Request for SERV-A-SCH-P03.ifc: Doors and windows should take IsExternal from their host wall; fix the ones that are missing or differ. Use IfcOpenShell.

First a look at what the model holds.

```python
import ifcopenshell
import ifcopenshell.util.element

model = ifcopenshell.open("SERV-A-SCH-P03.ifc")
print(model.schema)
seen = {}
for e in model.by_type("IfcDoor") + model.by_type("IfcWindow"):
    if not e.FillsVoids:
        continue
    host = e.FillsVoids[0].RelatingOpeningElement.VoidsElements[0].RelatingBuildingElement
    own = ifcopenshell.util.element.get_pset(e, f"Pset_{e.is_a()[3:].removesuffix('StandardCase')}Common", "IsExternal")
    wall = ifcopenshell.util.element.get_pset(host, "Pset_WallCommon", "IsExternal")
    seen[e.is_a(), own, wall] = seen.get((e.is_a(), own, wall), 0) + 1
for (cls, own, wall), count in sorted(seen.items(), key=str):
    print(count, cls, "IsExternal:", own, "| host wall:", wall)
```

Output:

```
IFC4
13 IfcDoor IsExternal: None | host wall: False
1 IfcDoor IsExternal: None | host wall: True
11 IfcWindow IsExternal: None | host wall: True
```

```python
import ifcopenshell
import ifcopenshell.api.pset
import ifcopenshell.util.element

model = ifcopenshell.open("SERV-A-SCH-P03.ifc")

count = 0
for ifc_class, pset_name in (("IfcDoor", "Pset_DoorCommon"), ("IfcWindow", "Pset_WindowCommon")):
    for e in model.by_type(ifc_class):
        if not e.FillsVoids:
            continue
        host = e.FillsVoids[0].RelatingOpeningElement.VoidsElements[0].RelatingBuildingElement
        external = ifcopenshell.util.element.get_pset(host, "Pset_WallCommon", "IsExternal")
        if external is None or ifcopenshell.util.element.get_pset(e, pset_name, "IsExternal") == external:
            continue
        pset = ifcopenshell.api.pset.add_pset(model, product=e, name=pset_name)
        ifcopenshell.api.pset.edit_pset(model, pset=pset, properties={"IsExternal": external})
        count += 1

print(count, "updated")

model.write("SERV-A-SCH-P03_updated.ifc")
```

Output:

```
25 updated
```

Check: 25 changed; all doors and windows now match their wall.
